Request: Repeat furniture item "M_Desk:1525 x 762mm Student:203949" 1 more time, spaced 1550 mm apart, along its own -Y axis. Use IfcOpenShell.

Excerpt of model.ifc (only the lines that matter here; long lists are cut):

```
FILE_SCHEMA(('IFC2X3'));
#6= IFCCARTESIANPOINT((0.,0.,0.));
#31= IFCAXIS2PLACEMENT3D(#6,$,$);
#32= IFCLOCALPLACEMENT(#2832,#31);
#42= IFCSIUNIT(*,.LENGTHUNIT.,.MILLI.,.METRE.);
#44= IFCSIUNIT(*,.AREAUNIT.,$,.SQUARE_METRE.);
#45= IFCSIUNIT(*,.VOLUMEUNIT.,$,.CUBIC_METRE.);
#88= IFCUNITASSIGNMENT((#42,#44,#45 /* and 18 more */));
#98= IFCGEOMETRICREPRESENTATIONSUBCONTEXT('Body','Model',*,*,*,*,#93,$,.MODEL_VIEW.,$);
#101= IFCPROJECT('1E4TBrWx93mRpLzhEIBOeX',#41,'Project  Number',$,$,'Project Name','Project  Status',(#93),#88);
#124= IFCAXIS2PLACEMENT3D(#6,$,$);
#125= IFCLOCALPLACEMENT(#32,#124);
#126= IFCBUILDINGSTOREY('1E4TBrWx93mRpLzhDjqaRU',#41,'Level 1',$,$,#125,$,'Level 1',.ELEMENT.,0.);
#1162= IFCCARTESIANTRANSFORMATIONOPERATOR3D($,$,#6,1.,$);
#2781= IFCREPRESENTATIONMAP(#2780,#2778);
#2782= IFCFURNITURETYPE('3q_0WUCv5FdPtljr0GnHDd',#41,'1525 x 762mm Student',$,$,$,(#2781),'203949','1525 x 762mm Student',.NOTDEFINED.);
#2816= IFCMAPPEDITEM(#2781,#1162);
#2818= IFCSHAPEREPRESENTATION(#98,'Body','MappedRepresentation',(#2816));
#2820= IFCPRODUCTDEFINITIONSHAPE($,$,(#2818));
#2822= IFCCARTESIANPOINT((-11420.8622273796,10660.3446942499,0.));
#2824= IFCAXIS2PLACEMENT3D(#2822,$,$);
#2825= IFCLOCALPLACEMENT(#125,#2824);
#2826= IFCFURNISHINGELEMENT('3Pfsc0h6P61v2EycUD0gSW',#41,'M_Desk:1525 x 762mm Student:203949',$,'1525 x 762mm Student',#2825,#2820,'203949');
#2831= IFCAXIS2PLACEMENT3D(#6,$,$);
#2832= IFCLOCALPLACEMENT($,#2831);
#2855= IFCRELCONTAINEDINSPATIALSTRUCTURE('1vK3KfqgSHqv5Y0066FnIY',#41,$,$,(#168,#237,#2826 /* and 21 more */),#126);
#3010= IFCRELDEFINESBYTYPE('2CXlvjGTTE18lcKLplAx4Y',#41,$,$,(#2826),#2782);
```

```python
import ifcopenshell
import ifcopenshell.api.geometry
import ifcopenshell.api.root
import ifcopenshell.util.element
import ifcopenshell.util.placement
import ifcopenshell.util.unit

model = ifcopenshell.open("model.ifc")
unit_scale = ifcopenshell.util.unit.calculate_unit_scale(model)

source = model.by_guid("3Pfsc0h6P61v2EycUD0gSW")
base = ifcopenshell.util.placement.get_local_placement(source.ObjectPlacement)
step = -base[:3, 1] * 1.55 / unit_scale

for i in range(1, 2):
    copy = ifcopenshell.api.root.copy_class(model, product=source)
    copy.Representation = ifcopenshell.util.element.copy_deep(
        model, source.Representation, exclude=["IfcGeometricRepresentationContext", "IfcRepresentationMap"]
    )
    copy.Name = "M_Desk:1525 x 762mm Student"
    copy.Tag = None
    matrix = base.copy()
    matrix[:3, 3] += i * step
    print("added at", matrix[:3, 3].round(3) + 0.0)
    ifcopenshell.api.geometry.edit_object_placement(model, product=copy, matrix=matrix, is_si=False)

model.write("model-out.ifc")
```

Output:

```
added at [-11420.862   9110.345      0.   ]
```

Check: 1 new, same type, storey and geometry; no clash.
